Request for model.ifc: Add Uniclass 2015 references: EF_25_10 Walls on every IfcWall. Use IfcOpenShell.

First a look at what the model holds.

```python
import ifcopenshell

model = ifcopenshell.open("model.ifc")
print(model.schema)
print("classifications:", [c.Name for c in model.by_type("IfcClassification")])
for ifc_class in ("IfcDoor", "IfcRoof", "IfcStair", "IfcWall", "IfcWindow"):
    print(ifc_class, len(model.by_type(ifc_class)))
```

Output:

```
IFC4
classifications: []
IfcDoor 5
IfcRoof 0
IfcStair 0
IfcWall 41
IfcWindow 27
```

```python
import ifcopenshell
import ifcopenshell.api.classification

model = ifcopenshell.open("model.ifc")

system = ifcopenshell.api.classification.add_classification(model, classification="Uniclass 2015")

codes = {
    "IfcWall": ("EF_25_10", "Walls"),
}
for ifc_class, (code, name) in codes.items():
    products = model.by_type(ifc_class)
    ifcopenshell.api.classification.add_reference(
        model, products=products, classification=system, identification=code, name=name
    )
    print(code, len(products))

model.write("model_rev.ifc")
```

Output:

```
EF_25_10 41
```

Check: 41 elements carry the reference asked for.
